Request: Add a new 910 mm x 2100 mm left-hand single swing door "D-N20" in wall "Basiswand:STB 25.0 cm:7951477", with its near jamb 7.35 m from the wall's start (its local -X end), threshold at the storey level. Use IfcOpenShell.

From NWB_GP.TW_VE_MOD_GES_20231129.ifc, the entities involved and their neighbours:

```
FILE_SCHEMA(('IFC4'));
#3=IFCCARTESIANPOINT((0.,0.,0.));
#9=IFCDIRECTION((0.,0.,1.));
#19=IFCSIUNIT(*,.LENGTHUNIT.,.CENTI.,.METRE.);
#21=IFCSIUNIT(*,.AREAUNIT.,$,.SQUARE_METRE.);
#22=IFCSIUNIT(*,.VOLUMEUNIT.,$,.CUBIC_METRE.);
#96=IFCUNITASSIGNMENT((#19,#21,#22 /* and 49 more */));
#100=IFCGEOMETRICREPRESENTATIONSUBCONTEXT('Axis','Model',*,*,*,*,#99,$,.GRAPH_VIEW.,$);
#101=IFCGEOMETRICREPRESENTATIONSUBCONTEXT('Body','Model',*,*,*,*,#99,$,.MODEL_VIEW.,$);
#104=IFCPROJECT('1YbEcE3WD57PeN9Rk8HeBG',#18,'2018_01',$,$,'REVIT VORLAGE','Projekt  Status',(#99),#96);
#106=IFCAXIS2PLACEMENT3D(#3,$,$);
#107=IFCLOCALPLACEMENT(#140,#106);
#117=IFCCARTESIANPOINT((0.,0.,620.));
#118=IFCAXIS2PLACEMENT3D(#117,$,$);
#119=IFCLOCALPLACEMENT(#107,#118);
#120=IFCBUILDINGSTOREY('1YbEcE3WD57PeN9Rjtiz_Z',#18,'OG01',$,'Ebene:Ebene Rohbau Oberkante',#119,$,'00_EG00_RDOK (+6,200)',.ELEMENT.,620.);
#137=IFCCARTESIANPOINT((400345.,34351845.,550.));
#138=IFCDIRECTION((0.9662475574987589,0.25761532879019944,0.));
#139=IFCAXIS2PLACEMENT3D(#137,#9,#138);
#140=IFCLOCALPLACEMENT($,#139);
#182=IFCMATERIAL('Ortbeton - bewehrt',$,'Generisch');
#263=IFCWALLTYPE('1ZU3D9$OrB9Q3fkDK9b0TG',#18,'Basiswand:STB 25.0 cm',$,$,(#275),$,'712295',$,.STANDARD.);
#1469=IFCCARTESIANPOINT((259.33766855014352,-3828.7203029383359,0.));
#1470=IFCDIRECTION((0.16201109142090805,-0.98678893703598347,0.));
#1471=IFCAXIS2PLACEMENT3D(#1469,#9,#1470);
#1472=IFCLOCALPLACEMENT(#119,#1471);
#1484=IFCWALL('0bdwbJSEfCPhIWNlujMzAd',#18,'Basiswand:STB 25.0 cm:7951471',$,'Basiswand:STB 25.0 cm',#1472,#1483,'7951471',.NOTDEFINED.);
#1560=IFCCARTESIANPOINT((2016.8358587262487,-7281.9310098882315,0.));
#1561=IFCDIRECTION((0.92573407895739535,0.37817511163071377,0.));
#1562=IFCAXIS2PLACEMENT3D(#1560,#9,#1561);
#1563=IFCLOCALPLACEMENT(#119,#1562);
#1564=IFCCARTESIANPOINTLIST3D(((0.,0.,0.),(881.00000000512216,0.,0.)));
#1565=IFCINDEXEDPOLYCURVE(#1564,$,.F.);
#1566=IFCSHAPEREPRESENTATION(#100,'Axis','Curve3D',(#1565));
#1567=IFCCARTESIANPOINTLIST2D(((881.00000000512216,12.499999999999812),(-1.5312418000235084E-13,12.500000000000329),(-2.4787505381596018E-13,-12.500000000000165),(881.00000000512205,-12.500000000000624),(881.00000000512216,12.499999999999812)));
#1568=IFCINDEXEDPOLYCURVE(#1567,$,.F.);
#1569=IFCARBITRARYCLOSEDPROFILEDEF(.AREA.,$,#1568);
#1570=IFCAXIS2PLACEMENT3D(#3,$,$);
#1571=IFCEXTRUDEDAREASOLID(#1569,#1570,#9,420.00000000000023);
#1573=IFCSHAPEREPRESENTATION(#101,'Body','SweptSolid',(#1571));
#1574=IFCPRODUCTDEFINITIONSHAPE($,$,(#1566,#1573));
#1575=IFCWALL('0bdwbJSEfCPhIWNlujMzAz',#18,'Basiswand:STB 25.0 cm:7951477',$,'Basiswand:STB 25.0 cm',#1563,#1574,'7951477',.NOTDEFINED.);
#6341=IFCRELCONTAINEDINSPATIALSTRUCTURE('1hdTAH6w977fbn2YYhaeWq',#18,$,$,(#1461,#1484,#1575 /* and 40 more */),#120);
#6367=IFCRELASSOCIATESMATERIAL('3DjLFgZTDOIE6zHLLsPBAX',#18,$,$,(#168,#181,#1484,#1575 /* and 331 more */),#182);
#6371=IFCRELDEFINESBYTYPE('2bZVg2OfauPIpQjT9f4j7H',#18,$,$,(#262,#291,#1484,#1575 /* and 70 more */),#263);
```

```python
import numpy as np
import ifcopenshell
import ifcopenshell.api.feature
import ifcopenshell.api.geometry
import ifcopenshell.api.root
import ifcopenshell.api.spatial
import ifcopenshell.geom
import ifcopenshell.util.element
import ifcopenshell.util.placement
import ifcopenshell.util.representation
import ifcopenshell.util.shape
import ifcopenshell.util.unit

model = ifcopenshell.open("NWB_GP.TW_VE_MOD_GES_20231129.ifc")
unit_scale = ifcopenshell.util.unit.calculate_unit_scale(model)
settings = ifcopenshell.geom.settings()


def volume(element):
    """Net volume in cubic metres, openings subtracted."""
    shape = ifcopenshell.geom.create_shape(settings, element)
    return ifcopenshell.util.shape.get_volume(shape.geometry)


wall = model.by_id(1575)
storey = ifcopenshell.util.element.get_container(wall, ifc_class="IfcBuildingStorey")
context = ifcopenshell.util.representation.get_context(model, "Model", "Body", "MODEL_VIEW")
before = volume(wall)

width, height, from_end, sill = 0.91, 2.1, 7.35, 0.0  # metres

# The wall runs along its own X axis, and the end named is its -X end.
wall_shape = ifcopenshell.geom.create_shape(settings, wall)
x, y, z = ifcopenshell.util.shape.get_vertices(wall_shape.geometry).T
start = x.min() + from_end
face, thickness = float(y.min()), float(y.max() - y.min())
wall_matrix = ifcopenshell.util.placement.get_local_placement(wall.ObjectPlacement)
level = ifcopenshell.util.placement.get_local_placement(storey.ObjectPlacement)[2, 3]


def in_wall(x, y):
    """Placement at x, y metres in the wall's axes, at sill height."""
    matrix = wall_matrix.copy()
    matrix[:, 3] = wall_matrix @ np.array([x / unit_scale, y / unit_scale, 0.0, 1.0])
    matrix[2, 3] = level + sill / unit_scale
    return matrix


# Opening: a box that overshoots both wall faces by 50 mm.
opening = ifcopenshell.api.root.create_entity(model, ifc_class="IfcOpeningElement", predefined_type="OPENING")
box = ifcopenshell.api.geometry.add_wall_representation(
    model, context=context, length=width, height=height, thickness=thickness + 0.1
)
ifcopenshell.api.geometry.assign_representation(model, product=opening, representation=box)
ifcopenshell.api.geometry.edit_object_placement(model, product=opening, matrix=in_wall(start, face - 0.05), is_si=False)
ifcopenshell.api.feature.add_feature(model, feature=opening, element=wall)

door = ifcopenshell.api.root.create_entity(model, ifc_class="IfcDoor", name="D-N20", predefined_type="DOOR")
door.OverallWidth, door.OverallHeight = width / unit_scale, height / unit_scale
door.OperationType = "SINGLE_SWING_LEFT"
body = ifcopenshell.api.geometry.add_door_representation(
    model,
    context=context,
    overall_width=door.OverallWidth,
    overall_height=door.OverallHeight,
    operation_type="SINGLE_SWING_LEFT",
    lining_properties={"LiningDepth": thickness / unit_scale, "ThresholdDepth": thickness / unit_scale},
)
ifcopenshell.api.geometry.assign_representation(model, product=door, representation=body)
ifcopenshell.api.spatial.assign_container(model, products=[door], relating_structure=storey)
ifcopenshell.api.feature.add_filling(model, opening=opening, element=door)

# The lining spans the wall, so the door starts at the wall face.
ifcopenshell.api.geometry.edit_object_placement(model, product=door, matrix=in_wall(start, face), is_si=False)

after = volume(wall)

print(f"wall volume {before:.3f} -> {after:.3f} m3")

model.write("NWB_GP.TW_VE_MOD_GES_20231129-out.ifc")
```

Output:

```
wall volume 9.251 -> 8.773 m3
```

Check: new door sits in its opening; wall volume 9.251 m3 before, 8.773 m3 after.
